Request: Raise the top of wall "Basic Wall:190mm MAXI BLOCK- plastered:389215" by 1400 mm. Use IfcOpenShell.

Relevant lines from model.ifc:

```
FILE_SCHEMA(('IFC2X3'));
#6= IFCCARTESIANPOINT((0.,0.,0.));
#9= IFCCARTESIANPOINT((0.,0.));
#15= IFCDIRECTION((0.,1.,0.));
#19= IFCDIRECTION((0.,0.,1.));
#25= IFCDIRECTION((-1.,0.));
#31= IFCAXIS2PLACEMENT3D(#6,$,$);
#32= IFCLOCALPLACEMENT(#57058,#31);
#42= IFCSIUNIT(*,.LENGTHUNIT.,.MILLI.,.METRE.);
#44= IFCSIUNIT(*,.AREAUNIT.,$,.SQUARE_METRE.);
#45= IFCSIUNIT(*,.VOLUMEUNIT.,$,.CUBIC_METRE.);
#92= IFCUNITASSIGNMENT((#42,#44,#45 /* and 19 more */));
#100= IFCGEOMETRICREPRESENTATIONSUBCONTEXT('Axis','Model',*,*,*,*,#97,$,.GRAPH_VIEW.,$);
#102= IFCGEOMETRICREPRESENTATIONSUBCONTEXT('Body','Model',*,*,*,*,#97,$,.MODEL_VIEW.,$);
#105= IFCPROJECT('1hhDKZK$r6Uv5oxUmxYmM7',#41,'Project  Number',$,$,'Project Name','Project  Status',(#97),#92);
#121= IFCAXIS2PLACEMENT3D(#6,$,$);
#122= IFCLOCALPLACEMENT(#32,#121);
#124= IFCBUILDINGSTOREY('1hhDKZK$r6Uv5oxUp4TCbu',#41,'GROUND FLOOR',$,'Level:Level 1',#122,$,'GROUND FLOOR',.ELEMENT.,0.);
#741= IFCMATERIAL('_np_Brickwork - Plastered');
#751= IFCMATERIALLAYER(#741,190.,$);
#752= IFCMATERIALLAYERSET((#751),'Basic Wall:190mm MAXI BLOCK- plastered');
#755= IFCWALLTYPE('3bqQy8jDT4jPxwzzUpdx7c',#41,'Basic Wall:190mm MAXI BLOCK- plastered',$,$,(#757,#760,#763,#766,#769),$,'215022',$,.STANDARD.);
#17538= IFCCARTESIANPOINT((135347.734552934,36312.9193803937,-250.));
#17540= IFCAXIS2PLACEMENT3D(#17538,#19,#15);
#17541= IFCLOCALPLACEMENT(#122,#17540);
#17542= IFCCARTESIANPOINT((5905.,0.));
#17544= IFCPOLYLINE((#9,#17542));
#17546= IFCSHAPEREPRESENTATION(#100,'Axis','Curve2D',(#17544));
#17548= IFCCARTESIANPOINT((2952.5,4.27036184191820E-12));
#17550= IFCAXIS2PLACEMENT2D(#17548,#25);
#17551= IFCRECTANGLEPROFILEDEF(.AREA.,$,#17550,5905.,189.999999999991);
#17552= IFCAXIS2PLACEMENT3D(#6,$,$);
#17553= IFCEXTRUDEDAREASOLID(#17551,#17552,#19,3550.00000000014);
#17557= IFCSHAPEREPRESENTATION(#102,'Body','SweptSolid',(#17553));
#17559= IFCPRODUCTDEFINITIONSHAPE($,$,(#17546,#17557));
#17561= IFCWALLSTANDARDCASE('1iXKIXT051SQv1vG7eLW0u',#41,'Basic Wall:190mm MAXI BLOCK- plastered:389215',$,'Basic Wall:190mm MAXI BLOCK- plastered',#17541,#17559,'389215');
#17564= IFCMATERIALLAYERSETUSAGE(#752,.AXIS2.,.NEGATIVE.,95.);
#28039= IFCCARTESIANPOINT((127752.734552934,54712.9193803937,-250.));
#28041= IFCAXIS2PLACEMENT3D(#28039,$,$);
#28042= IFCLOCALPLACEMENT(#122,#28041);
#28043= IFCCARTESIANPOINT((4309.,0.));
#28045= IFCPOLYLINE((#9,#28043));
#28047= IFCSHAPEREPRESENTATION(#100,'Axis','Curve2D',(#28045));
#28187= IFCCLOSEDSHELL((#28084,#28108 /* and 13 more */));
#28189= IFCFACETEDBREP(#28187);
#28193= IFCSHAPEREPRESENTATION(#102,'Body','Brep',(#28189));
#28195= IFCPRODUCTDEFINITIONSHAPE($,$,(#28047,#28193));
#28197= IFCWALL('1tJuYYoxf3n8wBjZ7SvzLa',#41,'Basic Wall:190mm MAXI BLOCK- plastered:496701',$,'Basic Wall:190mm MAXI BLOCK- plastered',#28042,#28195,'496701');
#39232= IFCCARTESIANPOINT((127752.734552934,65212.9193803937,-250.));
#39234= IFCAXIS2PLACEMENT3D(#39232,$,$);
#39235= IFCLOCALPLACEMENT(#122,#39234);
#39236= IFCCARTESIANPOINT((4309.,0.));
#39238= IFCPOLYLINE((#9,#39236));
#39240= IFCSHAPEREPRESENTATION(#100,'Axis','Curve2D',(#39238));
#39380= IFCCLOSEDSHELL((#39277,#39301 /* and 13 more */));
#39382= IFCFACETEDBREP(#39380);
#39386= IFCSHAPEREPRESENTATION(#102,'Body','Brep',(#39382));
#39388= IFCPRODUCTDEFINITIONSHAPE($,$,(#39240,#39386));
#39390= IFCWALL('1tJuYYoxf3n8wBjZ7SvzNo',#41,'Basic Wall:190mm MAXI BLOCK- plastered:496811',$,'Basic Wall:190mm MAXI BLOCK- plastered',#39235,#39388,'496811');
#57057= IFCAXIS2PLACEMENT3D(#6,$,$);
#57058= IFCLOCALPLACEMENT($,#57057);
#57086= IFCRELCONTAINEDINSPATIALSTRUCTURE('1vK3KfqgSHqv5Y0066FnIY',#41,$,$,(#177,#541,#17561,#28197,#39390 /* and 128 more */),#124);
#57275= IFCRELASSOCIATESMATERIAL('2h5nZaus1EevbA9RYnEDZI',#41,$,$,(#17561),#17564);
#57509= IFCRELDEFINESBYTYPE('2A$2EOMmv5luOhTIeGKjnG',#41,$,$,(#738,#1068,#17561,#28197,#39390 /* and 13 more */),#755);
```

```python
import ifcopenshell
import ifcopenshell.geom
import ifcopenshell.util.representation
import ifcopenshell.util.shape
import ifcopenshell.util.unit

model = ifcopenshell.open("model.ifc")
unit_scale = ifcopenshell.util.unit.calculate_unit_scale(model)
settings = ifcopenshell.geom.settings()


def volume(element):
    """Net volume in cubic metres, openings subtracted."""
    shape = ifcopenshell.geom.create_shape(settings, element)
    return ifcopenshell.util.shape.get_volume(shape.geometry)


wall = model.by_guid("1iXKIXT051SQv1vG7eLW0u")
before = volume(wall)

body = ifcopenshell.util.representation.get_representation(wall, "Model", "Body")
solid = body.Items[0]
old_height = solid.Depth
solid.Depth += 1.4 / unit_scale
after = volume(wall)

print(f"height {old_height:g} -> {solid.Depth:g}, volume {before:.3f} -> {after:.3f} m3")

model.write("model-out.ifc")
```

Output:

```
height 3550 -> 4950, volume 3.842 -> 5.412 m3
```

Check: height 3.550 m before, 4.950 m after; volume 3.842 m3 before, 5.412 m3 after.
